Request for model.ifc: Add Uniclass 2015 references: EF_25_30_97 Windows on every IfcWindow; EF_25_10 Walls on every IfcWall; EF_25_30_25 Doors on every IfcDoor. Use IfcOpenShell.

First a look at what the model holds.

```python
import ifcopenshell

model = ifcopenshell.open("model.ifc")
print(model.schema)
print("classifications:", [c.Name for c in model.by_type("IfcClassification")])
for ifc_class in ("IfcDoor", "IfcRoof", "IfcStair", "IfcWall", "IfcWindow"):
    print(ifc_class, len(model.by_type(ifc_class)))
```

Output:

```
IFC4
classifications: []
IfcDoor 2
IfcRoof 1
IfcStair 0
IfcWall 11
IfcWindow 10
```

```python
import ifcopenshell
import ifcopenshell.api.classification

model = ifcopenshell.open("model.ifc")

system = ifcopenshell.api.classification.add_classification(model, classification="Uniclass 2015")

codes = {
    "IfcWindow": ("EF_25_30_97", "Windows"),
    "IfcWall": ("EF_25_10", "Walls"),
    "IfcDoor": ("EF_25_30_25", "Doors"),
}
for ifc_class, (code, name) in codes.items():
    products = model.by_type(ifc_class)
    ifcopenshell.api.classification.add_reference(
        model, products=products, classification=system, identification=code, name=name
    )
    print(code, len(products))

model.write("model_updated.ifc")
```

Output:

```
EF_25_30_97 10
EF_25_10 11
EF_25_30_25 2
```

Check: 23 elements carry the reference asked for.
